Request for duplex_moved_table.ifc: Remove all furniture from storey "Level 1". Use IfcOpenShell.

First a look at what the model holds.

```python
import ifcopenshell
import ifcopenshell.util.element

model = ifcopenshell.open("duplex_moved_table.ifc")
print(model.schema)
storey = next(s for s in model.by_type("IfcBuildingStorey") if s.Name == "Level 1")
furniture = [e for e in ifcopenshell.util.element.get_decomposition(storey) if e.is_a("IfcFurnishingElement")]
seen = {}
for e in furniture:
    element_type = ifcopenshell.util.element.get_type(e)
    name = element_type.Name if element_type not in (None, e) else None
    seen[name] = seen.get(name, 0) + 1
for name, count in sorted(seen.items(), key=str):
    print(count, "x", name)
```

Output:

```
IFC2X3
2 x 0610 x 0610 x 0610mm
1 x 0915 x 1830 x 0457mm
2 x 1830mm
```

```python
import ifcopenshell
import ifcopenshell.api.root
import ifcopenshell.util.element

model = ifcopenshell.open("duplex_moved_table.ifc")

storey = next(s for s in model.by_type("IfcBuildingStorey") if s.Name == "Level 1")
furniture = [e for e in ifcopenshell.util.element.get_decomposition(storey) if e.is_a("IfcFurnishingElement")]

for e in furniture:
    ifcopenshell.api.root.remove_product(model, product=e)
print(len(furniture), "removed")

model.write("duplex_moved_table_rev.ifc")
```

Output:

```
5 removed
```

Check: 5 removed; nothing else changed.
